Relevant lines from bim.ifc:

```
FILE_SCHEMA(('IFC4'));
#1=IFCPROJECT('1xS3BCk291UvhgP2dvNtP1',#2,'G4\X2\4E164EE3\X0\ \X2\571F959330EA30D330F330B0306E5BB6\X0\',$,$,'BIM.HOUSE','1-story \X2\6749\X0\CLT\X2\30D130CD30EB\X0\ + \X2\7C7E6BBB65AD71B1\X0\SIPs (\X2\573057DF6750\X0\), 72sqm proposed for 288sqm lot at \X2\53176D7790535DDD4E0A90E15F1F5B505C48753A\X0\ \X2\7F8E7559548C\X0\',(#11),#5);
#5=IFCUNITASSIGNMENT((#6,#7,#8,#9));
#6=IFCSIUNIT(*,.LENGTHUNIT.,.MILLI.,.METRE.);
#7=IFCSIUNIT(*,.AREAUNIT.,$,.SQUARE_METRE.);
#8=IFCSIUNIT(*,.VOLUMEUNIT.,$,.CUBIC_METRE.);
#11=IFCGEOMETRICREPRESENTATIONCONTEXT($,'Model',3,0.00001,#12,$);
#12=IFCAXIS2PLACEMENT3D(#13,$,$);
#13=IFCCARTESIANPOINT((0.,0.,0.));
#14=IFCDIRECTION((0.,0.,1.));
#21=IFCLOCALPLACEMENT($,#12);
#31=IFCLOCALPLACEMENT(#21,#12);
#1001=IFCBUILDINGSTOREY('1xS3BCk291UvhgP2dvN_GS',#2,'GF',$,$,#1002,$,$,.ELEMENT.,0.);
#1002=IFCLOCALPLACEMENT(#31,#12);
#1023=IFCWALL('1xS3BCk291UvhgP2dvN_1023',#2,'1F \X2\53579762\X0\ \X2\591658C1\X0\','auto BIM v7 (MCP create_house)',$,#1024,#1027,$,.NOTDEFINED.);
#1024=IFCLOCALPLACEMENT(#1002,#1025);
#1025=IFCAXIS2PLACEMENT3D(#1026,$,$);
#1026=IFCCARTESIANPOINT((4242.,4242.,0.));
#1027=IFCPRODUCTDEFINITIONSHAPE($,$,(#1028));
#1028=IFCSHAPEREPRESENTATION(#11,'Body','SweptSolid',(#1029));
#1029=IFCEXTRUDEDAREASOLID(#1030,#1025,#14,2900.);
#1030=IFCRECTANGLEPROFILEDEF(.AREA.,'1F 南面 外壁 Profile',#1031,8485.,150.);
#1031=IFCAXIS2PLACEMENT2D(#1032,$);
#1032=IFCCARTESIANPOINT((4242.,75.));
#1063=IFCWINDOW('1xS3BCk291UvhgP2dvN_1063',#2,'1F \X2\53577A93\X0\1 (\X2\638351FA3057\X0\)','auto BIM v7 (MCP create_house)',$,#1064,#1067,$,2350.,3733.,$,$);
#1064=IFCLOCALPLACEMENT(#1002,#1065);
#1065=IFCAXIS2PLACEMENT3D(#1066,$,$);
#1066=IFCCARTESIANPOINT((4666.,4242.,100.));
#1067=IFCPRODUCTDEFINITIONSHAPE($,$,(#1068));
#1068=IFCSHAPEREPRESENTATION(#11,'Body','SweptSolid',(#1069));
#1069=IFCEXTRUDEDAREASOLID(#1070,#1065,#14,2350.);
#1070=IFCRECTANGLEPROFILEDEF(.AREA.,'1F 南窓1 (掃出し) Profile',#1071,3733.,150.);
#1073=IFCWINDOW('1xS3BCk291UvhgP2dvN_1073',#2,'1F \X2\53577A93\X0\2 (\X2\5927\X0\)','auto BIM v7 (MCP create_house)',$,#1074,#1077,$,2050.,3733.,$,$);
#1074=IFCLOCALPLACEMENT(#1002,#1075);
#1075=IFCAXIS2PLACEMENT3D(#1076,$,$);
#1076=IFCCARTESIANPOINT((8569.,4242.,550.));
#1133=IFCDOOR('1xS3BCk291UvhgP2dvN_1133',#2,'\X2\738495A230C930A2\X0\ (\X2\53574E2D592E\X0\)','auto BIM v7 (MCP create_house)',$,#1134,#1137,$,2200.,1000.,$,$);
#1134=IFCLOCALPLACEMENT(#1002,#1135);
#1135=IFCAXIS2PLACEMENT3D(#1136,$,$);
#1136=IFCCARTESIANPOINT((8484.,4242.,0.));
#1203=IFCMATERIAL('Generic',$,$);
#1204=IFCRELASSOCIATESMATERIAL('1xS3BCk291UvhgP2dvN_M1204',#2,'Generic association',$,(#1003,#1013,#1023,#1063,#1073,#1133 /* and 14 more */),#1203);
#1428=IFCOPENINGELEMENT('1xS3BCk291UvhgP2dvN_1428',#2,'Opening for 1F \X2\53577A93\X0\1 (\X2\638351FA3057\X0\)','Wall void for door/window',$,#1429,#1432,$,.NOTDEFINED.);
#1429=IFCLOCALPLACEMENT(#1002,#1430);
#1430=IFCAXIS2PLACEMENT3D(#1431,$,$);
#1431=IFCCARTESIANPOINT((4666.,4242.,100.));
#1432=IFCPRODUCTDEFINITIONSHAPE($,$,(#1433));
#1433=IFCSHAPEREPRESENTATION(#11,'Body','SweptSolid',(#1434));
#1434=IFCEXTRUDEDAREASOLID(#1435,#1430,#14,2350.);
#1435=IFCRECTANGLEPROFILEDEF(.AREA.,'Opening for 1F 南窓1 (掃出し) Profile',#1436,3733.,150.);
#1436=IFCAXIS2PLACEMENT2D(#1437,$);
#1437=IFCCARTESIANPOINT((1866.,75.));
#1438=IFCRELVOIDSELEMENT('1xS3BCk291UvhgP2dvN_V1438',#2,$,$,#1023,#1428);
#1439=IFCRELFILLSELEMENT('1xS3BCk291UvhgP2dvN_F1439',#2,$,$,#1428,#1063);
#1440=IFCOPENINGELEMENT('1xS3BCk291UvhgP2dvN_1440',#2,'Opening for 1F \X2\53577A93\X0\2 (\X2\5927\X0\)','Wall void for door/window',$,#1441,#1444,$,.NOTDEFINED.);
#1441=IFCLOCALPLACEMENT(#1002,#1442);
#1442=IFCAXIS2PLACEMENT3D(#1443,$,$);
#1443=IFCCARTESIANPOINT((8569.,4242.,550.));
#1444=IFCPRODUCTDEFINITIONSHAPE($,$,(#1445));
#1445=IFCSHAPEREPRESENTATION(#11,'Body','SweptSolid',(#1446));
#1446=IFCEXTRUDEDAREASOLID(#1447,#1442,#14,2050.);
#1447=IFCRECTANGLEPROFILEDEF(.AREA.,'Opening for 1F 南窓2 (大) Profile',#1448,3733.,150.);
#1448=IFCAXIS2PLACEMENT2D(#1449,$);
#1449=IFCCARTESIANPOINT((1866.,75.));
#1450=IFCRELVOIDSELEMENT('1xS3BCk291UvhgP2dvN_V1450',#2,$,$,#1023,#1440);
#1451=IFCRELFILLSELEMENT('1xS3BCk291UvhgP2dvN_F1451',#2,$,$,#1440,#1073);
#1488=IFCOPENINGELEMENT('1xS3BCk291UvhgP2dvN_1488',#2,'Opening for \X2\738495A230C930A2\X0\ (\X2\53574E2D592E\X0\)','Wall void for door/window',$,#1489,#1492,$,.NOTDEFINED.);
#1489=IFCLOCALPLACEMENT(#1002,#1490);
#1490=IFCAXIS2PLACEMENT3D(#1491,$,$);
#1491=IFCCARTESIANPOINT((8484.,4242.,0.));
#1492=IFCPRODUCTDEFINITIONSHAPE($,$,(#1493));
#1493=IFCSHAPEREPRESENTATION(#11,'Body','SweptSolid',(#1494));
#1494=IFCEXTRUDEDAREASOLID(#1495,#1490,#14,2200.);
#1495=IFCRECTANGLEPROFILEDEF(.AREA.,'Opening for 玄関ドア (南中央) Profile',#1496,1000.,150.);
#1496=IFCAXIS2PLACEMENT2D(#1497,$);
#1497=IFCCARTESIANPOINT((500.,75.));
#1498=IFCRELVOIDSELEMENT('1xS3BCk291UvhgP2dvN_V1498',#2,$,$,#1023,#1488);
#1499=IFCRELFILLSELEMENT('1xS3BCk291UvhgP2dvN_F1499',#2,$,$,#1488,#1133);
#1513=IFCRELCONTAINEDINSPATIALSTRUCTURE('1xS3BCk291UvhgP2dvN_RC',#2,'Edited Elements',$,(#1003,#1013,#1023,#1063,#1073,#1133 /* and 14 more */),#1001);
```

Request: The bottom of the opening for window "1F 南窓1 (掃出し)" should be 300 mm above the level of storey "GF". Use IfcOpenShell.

```python
import numpy as np
import ifcopenshell
import ifcopenshell.api.geometry
import ifcopenshell.geom
import ifcopenshell.util.element
import ifcopenshell.util.placement
import ifcopenshell.util.shape
import ifcopenshell.util.unit

model = ifcopenshell.open("bim.ifc")
unit_scale = ifcopenshell.util.unit.calculate_unit_scale(model)

window = model.by_id(1063)
opening = window.FillsVoids[0].RelatingOpeningElement
storey = ifcopenshell.util.element.get_container(window, ifc_class="IfcBuildingStorey")
level = ifcopenshell.util.placement.get_local_placement(storey.ObjectPlacement)[2, 3]

# The opening's origin need not be at the sill, so measure its lowest point.
shape = ifcopenshell.geom.create_shape(ifcopenshell.geom.settings(), opening)
bottom = ifcopenshell.util.shape.get_shape_bottom_elevation(shape, shape.geometry) / unit_scale
dz = level + 0.3 / unit_scale - bottom

shift = np.array([0.0, 0.0, dz])
# The window is not placed relative to its opening, so move both.
for product in (opening, window):
    matrix = ifcopenshell.util.placement.get_local_placement(product.ObjectPlacement)
    matrix[:3, 3] += shift
    ifcopenshell.api.geometry.edit_object_placement(model, product=product, matrix=matrix, is_si=False)

print(f"moved by {dz * unit_scale:+.3f} m")

model.write("bim_edited.ifc")
```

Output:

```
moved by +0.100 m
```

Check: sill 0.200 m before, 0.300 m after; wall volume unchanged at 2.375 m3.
